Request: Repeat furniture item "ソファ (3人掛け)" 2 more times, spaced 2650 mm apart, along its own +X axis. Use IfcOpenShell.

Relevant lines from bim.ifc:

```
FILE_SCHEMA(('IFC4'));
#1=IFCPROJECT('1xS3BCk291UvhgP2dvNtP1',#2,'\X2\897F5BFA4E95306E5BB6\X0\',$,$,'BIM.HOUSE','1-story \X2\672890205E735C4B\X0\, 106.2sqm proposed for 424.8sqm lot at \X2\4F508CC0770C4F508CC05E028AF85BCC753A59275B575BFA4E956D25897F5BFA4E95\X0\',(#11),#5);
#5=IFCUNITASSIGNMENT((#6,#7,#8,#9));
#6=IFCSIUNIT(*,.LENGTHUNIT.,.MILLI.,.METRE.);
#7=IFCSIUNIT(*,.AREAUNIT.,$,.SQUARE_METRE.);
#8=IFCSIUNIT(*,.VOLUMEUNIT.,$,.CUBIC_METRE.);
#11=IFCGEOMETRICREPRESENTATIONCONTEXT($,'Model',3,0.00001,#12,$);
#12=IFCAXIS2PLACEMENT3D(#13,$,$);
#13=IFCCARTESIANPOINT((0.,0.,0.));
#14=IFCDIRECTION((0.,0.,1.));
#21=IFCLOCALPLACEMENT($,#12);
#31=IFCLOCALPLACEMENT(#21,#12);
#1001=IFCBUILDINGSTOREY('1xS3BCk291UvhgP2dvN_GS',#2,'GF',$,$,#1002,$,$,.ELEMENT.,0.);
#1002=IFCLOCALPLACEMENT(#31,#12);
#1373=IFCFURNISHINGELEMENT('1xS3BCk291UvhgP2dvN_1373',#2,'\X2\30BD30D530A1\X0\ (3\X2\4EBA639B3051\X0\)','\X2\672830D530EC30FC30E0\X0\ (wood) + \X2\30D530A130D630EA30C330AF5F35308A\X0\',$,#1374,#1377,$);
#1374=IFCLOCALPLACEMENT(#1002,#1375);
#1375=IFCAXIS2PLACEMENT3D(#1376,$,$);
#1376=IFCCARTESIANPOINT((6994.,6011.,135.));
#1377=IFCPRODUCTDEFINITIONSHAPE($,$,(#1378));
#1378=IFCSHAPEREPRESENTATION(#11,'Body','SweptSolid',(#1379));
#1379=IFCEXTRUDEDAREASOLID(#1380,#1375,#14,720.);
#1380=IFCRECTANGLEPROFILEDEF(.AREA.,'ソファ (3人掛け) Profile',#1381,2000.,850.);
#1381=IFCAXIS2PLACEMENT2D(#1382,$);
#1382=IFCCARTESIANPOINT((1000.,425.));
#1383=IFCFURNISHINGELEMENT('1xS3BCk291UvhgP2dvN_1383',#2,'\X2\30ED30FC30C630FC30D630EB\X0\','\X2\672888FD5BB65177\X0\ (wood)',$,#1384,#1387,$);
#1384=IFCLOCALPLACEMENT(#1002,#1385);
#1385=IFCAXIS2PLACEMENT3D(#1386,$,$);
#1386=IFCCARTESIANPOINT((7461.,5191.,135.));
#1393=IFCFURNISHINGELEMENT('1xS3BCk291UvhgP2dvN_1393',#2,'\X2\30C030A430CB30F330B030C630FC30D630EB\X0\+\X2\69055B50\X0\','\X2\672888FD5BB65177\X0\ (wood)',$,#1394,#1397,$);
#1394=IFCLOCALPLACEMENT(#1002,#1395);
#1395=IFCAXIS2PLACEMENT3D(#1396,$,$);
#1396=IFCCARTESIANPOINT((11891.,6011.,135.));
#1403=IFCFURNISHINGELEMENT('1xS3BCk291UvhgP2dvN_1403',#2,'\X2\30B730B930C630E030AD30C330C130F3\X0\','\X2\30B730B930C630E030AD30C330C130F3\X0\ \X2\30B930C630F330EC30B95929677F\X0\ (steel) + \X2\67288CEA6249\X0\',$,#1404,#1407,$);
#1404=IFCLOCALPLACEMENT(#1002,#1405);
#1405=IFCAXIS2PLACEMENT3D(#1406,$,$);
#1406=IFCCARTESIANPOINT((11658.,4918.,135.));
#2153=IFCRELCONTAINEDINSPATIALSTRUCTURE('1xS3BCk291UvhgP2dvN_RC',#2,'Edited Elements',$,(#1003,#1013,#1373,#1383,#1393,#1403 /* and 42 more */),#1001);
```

```python
import ifcopenshell
import ifcopenshell.api.geometry
import ifcopenshell.api.root
import ifcopenshell.util.element
import ifcopenshell.util.placement

model = ifcopenshell.open("bim.ifc")


def reuse_history(source, copy):
    """copy_class also copies each property set's owner history, people and application; keep the originals."""
    for rel in copy.IsDefinedBy:
        if rel.is_a("IfcRelDefinesByProperties") and (history := rel.RelatingPropertyDefinition.OwnerHistory):
            rel.RelatingPropertyDefinition.OwnerHistory = source.OwnerHistory
            ifcopenshell.util.element.remove_deep2(model, history)


source = model.by_guid("1xS3BCk291UvhgP2dvN_1373")
base = ifcopenshell.util.placement.get_local_placement(source.ObjectPlacement)
step = base[:3, 0] * 2650.0

for i in range(1, 3):
    copy = ifcopenshell.api.root.copy_class(model, product=source)
    copy.Representation = ifcopenshell.util.element.copy_deep(
        model, source.Representation, exclude=["IfcGeometricRepresentationContext", "IfcRepresentationMap"]
    )
    reuse_history(source, copy)
    matrix = base.copy()
    matrix[:3, 3] += i * step
    print("added at", matrix[:3, 3].round(3) + 0.0)
    ifcopenshell.api.geometry.edit_object_placement(model, product=copy, matrix=matrix, is_si=False)

model.write("bim_rev.ifc")
```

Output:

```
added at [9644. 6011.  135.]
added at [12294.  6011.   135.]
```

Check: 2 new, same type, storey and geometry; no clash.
